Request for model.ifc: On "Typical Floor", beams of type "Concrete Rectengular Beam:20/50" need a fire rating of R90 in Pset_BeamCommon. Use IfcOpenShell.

First a look at what the model holds.

```python
import ifcopenshell
import ifcopenshell.util.element

model = ifcopenshell.open("model.ifc")
print(model.schema)
storey = next(s for s in model.by_type("IfcBuildingStorey") if s.Name == "Typical Floor")
beams = [e for e in ifcopenshell.util.element.get_decomposition(storey) if e.is_a("IfcBeam")]
seen = {}
for e in beams:
    element_type = ifcopenshell.util.element.get_type(e)
    key = (element_type.Name if element_type != e and element_type else None, ifcopenshell.util.element.get_pset(e, "Pset_BeamCommon", "FireRating"))
    seen[key] = seen.get(key, 0) + 1
for (name, value), count in sorted(seen.items(), key=str):
    print(count, "x", name, "|", value)
```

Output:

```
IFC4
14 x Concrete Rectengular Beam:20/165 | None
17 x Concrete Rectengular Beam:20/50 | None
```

```python
import ifcopenshell
import ifcopenshell.api.pset
import ifcopenshell.util.element

model = ifcopenshell.open("model.ifc")

storey = next(s for s in model.by_type("IfcBuildingStorey") if s.Name == "Typical Floor")
beams = [e for e in ifcopenshell.util.element.get_decomposition(storey) if e.is_a("IfcBeam")]

count = 0
for e in beams:
    element_type = ifcopenshell.util.element.get_type(e)
    if element_type in (None, e) or element_type.Name != "Concrete Rectengular Beam:20/50":
        continue
    # add_pset returns the element's existing set when there is one.
    pset = ifcopenshell.api.pset.add_pset(model, product=e, name="Pset_BeamCommon")
    ifcopenshell.api.pset.edit_pset(model, pset=pset, properties={"FireRating": "R90"})
    count += 1

print(count, "beams updated")

model.write("model-out.ifc")
```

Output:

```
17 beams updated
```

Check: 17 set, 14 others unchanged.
